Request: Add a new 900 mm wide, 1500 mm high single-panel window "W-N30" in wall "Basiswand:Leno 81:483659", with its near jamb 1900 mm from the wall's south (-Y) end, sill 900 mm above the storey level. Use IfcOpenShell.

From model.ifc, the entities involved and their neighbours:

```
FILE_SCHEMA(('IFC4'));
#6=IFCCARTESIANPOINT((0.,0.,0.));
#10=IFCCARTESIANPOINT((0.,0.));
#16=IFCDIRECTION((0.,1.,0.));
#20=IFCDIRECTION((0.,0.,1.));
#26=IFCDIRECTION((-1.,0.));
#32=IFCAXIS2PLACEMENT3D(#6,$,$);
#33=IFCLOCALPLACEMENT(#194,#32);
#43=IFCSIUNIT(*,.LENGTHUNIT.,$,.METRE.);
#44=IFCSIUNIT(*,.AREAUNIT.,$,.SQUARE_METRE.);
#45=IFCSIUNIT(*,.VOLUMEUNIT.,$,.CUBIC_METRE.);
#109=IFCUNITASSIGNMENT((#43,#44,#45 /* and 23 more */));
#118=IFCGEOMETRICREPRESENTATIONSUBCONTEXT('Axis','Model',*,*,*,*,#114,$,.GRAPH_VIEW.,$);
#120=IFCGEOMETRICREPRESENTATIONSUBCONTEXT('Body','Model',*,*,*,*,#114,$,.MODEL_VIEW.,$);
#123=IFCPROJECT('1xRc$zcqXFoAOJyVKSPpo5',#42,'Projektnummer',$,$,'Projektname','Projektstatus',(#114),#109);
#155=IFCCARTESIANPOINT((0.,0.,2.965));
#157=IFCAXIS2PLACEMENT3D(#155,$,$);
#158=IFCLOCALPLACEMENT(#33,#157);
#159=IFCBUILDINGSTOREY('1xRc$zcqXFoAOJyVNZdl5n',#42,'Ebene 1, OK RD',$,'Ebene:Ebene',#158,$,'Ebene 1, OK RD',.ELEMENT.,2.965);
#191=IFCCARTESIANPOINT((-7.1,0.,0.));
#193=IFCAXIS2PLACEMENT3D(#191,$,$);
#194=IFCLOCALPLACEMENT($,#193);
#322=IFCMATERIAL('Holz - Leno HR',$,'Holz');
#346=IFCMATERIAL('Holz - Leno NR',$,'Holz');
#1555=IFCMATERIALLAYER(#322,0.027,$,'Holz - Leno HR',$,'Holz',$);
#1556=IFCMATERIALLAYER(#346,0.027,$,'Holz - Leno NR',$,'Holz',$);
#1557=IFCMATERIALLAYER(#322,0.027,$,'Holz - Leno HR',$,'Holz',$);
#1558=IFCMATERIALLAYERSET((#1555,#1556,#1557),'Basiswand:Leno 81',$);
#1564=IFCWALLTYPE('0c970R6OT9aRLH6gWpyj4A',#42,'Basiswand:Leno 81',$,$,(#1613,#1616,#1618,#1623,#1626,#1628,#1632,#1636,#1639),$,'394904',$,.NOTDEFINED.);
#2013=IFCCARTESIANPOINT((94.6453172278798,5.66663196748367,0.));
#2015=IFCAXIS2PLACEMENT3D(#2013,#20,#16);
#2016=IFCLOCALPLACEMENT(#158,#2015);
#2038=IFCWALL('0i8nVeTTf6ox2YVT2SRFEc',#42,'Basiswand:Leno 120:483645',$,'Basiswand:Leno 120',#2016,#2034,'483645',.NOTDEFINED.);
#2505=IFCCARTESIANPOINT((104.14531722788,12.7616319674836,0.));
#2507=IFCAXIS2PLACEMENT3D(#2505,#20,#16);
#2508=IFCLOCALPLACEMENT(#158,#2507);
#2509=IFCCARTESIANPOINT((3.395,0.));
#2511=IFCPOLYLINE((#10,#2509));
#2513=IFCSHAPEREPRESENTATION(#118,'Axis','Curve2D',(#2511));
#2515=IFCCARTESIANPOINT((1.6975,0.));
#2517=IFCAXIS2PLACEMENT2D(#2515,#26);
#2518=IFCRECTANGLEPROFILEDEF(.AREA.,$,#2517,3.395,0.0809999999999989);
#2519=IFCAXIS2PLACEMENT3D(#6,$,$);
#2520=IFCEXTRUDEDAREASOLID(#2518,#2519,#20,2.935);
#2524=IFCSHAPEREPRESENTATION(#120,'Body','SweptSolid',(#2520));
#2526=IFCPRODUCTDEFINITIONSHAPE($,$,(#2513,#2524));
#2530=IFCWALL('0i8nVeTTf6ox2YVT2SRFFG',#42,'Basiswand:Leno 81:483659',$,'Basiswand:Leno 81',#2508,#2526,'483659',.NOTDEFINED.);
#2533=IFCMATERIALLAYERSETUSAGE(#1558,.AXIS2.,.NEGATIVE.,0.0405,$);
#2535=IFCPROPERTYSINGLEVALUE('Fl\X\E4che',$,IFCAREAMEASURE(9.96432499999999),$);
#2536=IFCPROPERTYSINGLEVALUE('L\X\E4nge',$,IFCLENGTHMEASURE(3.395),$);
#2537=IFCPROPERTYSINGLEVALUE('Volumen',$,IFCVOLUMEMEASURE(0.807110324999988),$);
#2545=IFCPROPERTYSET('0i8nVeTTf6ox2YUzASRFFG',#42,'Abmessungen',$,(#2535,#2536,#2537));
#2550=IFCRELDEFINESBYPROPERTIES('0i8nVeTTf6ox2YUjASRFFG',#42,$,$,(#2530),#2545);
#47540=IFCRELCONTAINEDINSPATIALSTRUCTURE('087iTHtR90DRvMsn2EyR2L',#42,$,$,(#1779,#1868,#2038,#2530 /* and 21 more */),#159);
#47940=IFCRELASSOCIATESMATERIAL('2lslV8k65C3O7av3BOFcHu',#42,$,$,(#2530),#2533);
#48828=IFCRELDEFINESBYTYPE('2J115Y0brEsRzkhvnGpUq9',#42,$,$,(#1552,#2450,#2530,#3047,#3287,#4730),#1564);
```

```python
import numpy as np
import ifcopenshell
import ifcopenshell.api.feature
import ifcopenshell.api.geometry
import ifcopenshell.api.pset
import ifcopenshell.api.root
import ifcopenshell.api.spatial
import ifcopenshell.geom
import ifcopenshell.util.element
import ifcopenshell.util.placement
import ifcopenshell.util.representation
import ifcopenshell.util.shape
import ifcopenshell.util.unit

model = ifcopenshell.open("model.ifc")
unit_scale = ifcopenshell.util.unit.calculate_unit_scale(model)
area_scale = ifcopenshell.util.unit.calculate_unit_scale(model, "AREAUNIT")
volume_scale = ifcopenshell.util.unit.calculate_unit_scale(model, "VOLUMEUNIT")
settings = ifcopenshell.geom.settings()


def volume(element):
    """Net volume in cubic metres, openings subtracted."""
    shape = ifcopenshell.geom.create_shape(settings, element)
    return ifcopenshell.util.shape.get_volume(shape.geometry)


wall = model.by_id(2530)
storey = ifcopenshell.util.element.get_container(wall, ifc_class="IfcBuildingStorey")
context = ifcopenshell.util.representation.get_context(model, "Model", "Body", "MODEL_VIEW")
before = volume(wall)

width, height, from_end, sill = 0.9, 1.5, 1.9, 0.9  # metres

# The wall runs along its own X axis, and the end named is its -X end.
wall_shape = ifcopenshell.geom.create_shape(settings, wall)
x, y, z = ifcopenshell.util.shape.get_vertices(wall_shape.geometry).T
start = x.min() + from_end
face, thickness = float(y.min()), float(y.max() - y.min())
wall_matrix = ifcopenshell.util.placement.get_local_placement(wall.ObjectPlacement)
level = ifcopenshell.util.placement.get_local_placement(storey.ObjectPlacement)[2, 3]


def in_wall(x, y):
    """Placement at x, y metres in the wall's axes, at sill height."""
    matrix = wall_matrix.copy()
    matrix[:, 3] = wall_matrix @ np.array([x / unit_scale, y / unit_scale, 0.0, 1.0])
    matrix[2, 3] = level + sill / unit_scale
    return matrix


# Opening: a box that overshoots both wall faces by 50 mm.
opening = ifcopenshell.api.root.create_entity(model, ifc_class="IfcOpeningElement", predefined_type="OPENING")
box = ifcopenshell.api.geometry.add_wall_representation(
    model, context=context, length=width, height=height, thickness=thickness + 0.1
)
ifcopenshell.api.geometry.assign_representation(model, product=opening, representation=box)
ifcopenshell.api.geometry.edit_object_placement(model, product=opening, matrix=in_wall(start, face - 0.05), is_si=False)
ifcopenshell.api.feature.add_feature(model, feature=opening, element=wall)

window = ifcopenshell.api.root.create_entity(model, ifc_class="IfcWindow", name="W-N30", predefined_type="WINDOW")
window.OverallWidth, window.OverallHeight = width / unit_scale, height / unit_scale
window.PartitioningType = "SINGLE_PANEL"
body = ifcopenshell.api.geometry.add_window_representation(
    model,
    context=context,
    overall_width=window.OverallWidth,
    overall_height=window.OverallHeight,
    partition_type="SINGLE_PANEL",
)
ifcopenshell.api.geometry.assign_representation(model, product=window, representation=body)
ifcopenshell.api.spatial.assign_container(model, products=[window], relating_structure=storey)
ifcopenshell.api.feature.add_filling(model, opening=opening, element=window)

# Centre the window in the wall's thickness.
ifcopenshell.api.geometry.edit_object_placement(model, product=window, matrix=in_wall(start, face), is_si=False)
window_shape = ifcopenshell.geom.create_shape(settings, window)
depth = ifcopenshell.util.shape.get_vertices(window_shape.geometry)[:, 1]
offset = face + thickness / 2 - (depth.min() + depth.max()) / 2
ifcopenshell.api.geometry.edit_object_placement(model, product=window, matrix=in_wall(start, offset), is_si=False)

after = volume(wall)

# Update the wall's stored quantities.
pset = model.by_id(ifcopenshell.util.element.get_pset(wall, "Abmessungen", should_inherit=False)["id"])
ifcopenshell.api.pset.edit_pset(model, pset=pset, properties={
    "Fläche": model.create_entity("IfcAreaMeasure", after / thickness / area_scale),
    "Volumen": model.create_entity("IfcVolumeMeasure", after / volume_scale),
})

print(f"wall volume {before:.3f} -> {after:.3f} m3")

model.write("model_edited.ifc")
```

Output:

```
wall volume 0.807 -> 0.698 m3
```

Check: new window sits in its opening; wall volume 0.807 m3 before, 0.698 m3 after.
